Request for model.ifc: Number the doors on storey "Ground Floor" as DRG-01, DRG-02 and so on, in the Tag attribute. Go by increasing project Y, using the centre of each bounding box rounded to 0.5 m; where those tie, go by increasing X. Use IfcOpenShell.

First a look at what the model holds.

```python
import ifcopenshell
import ifcopenshell.util.element
import ifcopenshell.util.placement

model = ifcopenshell.open("model.ifc")
print(model.schema)
storey = next(s for s in model.by_type("IfcBuildingStorey") if s.Name == "Ground Floor")
doors = [e for e in ifcopenshell.util.element.get_decomposition(storey) if e.is_a("IfcDoor")]
for e in sorted(doors, key=lambda e: e.id()):
    origin = ifcopenshell.util.placement.get_local_placement(e.ObjectPlacement)[:3, 3]
    print(e.id(), e.Tag, e.Name, origin.round(2) + 0.0, sep=" | ")
```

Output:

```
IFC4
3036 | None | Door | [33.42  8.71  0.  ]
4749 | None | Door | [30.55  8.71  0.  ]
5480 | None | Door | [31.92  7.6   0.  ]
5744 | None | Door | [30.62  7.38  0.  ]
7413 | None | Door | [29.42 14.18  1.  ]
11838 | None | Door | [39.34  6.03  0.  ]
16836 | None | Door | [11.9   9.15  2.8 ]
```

```python
import ifcopenshell
import ifcopenshell.geom
import ifcopenshell.util.element
import ifcopenshell.util.shape

model = ifcopenshell.open("model.ifc")
settings = ifcopenshell.geom.settings()
settings.set("use-world-coords", True)


def centre(element):
    shape = ifcopenshell.geom.create_shape(settings, element)
    return ifcopenshell.util.shape.get_bbox_centroid(shape.geometry)


storey = next(s for s in model.by_type("IfcBuildingStorey") if s.Name == "Ground Floor")
doors = [e for e in ifcopenshell.util.element.get_decomposition(storey) if e.is_a("IfcDoor")]

# Insertion points can sit at a corner or the storey origin, so sort by the geometry (in metres).
centres = {e: centre(e) for e in doors}
doors.sort(key=lambda e: (round(centres[e][1] / 0.5), centres[e][0]))

for i, e in enumerate(doors, start=1):
    number = f"DRG-{i:02d}"
    e.Tag = number
    print(e.id(), number)

model.write("model_v2.ifc")
```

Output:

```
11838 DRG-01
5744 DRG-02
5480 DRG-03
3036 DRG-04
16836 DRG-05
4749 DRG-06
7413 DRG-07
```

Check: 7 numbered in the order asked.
